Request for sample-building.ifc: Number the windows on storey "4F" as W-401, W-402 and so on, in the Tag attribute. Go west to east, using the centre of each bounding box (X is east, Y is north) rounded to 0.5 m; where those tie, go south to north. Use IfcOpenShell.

First a look at what the model holds.

```python
import ifcopenshell
import ifcopenshell.util.element
import ifcopenshell.util.placement

model = ifcopenshell.open("sample-building.ifc")
print(model.schema)
storey = next(s for s in model.by_type("IfcBuildingStorey") if s.Name == "4F")
windows = [e for e in ifcopenshell.util.element.get_decomposition(storey) if e.is_a("IfcWindow")]
for e in sorted(windows, key=lambda e: e.id()):
    origin = ifcopenshell.util.placement.get_local_placement(e.ObjectPlacement)[:3, 3]
    print(e.id(), e.Tag, e.Name, origin.round(2) + 0.0, sep=" | ")
```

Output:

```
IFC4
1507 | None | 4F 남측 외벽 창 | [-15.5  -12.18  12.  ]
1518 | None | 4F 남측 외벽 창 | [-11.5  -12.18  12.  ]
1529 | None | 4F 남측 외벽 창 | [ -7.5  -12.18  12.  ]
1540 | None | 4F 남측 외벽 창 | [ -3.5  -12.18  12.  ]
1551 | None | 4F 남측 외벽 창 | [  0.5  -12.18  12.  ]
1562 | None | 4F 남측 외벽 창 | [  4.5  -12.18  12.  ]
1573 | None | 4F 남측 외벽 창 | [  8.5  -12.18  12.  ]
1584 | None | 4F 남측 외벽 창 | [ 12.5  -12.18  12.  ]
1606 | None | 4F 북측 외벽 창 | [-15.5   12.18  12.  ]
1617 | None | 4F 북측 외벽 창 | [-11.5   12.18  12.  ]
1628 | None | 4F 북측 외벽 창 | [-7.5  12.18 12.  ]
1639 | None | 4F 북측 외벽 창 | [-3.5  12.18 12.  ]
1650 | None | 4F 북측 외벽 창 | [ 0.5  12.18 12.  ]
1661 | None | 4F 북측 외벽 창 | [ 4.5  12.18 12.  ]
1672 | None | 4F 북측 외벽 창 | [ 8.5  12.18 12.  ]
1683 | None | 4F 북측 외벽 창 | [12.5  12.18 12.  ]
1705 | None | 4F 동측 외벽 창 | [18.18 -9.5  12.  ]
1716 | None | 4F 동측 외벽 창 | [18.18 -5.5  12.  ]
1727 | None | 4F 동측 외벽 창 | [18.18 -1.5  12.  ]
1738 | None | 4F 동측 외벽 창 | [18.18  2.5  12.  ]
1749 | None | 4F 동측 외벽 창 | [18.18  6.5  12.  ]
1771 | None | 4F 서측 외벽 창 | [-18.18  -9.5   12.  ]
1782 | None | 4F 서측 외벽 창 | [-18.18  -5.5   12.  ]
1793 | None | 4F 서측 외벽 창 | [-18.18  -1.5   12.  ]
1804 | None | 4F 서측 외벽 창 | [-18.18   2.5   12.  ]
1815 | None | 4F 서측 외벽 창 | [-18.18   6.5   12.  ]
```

```python
import ifcopenshell
import ifcopenshell.geom
import ifcopenshell.util.element
import ifcopenshell.util.shape

model = ifcopenshell.open("sample-building.ifc")
settings = ifcopenshell.geom.settings()
settings.set("use-world-coords", True)


def centre(element):
    shape = ifcopenshell.geom.create_shape(settings, element)
    return ifcopenshell.util.shape.get_bbox_centroid(shape.geometry)


storey = next(s for s in model.by_type("IfcBuildingStorey") if s.Name == "4F")
windows = [e for e in ifcopenshell.util.element.get_decomposition(storey) if e.is_a("IfcWindow")]

# Insertion points can sit at a corner or the storey origin, so sort by the geometry (in metres).
centres = {e: centre(e) for e in windows}
windows.sort(key=lambda e: (round(centres[e][0] / 0.5), centres[e][1]))

for i, e in enumerate(windows, start=1):
    number = f"W-4{i:02d}"
    e.Tag = number
    print(e.id(), number)

model.write("sample-building_rev.ifc")
```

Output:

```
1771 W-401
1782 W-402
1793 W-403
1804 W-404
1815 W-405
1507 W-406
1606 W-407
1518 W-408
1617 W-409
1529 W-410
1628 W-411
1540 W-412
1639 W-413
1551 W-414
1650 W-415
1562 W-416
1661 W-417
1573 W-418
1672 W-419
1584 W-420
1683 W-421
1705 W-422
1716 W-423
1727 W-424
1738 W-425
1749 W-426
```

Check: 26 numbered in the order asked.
